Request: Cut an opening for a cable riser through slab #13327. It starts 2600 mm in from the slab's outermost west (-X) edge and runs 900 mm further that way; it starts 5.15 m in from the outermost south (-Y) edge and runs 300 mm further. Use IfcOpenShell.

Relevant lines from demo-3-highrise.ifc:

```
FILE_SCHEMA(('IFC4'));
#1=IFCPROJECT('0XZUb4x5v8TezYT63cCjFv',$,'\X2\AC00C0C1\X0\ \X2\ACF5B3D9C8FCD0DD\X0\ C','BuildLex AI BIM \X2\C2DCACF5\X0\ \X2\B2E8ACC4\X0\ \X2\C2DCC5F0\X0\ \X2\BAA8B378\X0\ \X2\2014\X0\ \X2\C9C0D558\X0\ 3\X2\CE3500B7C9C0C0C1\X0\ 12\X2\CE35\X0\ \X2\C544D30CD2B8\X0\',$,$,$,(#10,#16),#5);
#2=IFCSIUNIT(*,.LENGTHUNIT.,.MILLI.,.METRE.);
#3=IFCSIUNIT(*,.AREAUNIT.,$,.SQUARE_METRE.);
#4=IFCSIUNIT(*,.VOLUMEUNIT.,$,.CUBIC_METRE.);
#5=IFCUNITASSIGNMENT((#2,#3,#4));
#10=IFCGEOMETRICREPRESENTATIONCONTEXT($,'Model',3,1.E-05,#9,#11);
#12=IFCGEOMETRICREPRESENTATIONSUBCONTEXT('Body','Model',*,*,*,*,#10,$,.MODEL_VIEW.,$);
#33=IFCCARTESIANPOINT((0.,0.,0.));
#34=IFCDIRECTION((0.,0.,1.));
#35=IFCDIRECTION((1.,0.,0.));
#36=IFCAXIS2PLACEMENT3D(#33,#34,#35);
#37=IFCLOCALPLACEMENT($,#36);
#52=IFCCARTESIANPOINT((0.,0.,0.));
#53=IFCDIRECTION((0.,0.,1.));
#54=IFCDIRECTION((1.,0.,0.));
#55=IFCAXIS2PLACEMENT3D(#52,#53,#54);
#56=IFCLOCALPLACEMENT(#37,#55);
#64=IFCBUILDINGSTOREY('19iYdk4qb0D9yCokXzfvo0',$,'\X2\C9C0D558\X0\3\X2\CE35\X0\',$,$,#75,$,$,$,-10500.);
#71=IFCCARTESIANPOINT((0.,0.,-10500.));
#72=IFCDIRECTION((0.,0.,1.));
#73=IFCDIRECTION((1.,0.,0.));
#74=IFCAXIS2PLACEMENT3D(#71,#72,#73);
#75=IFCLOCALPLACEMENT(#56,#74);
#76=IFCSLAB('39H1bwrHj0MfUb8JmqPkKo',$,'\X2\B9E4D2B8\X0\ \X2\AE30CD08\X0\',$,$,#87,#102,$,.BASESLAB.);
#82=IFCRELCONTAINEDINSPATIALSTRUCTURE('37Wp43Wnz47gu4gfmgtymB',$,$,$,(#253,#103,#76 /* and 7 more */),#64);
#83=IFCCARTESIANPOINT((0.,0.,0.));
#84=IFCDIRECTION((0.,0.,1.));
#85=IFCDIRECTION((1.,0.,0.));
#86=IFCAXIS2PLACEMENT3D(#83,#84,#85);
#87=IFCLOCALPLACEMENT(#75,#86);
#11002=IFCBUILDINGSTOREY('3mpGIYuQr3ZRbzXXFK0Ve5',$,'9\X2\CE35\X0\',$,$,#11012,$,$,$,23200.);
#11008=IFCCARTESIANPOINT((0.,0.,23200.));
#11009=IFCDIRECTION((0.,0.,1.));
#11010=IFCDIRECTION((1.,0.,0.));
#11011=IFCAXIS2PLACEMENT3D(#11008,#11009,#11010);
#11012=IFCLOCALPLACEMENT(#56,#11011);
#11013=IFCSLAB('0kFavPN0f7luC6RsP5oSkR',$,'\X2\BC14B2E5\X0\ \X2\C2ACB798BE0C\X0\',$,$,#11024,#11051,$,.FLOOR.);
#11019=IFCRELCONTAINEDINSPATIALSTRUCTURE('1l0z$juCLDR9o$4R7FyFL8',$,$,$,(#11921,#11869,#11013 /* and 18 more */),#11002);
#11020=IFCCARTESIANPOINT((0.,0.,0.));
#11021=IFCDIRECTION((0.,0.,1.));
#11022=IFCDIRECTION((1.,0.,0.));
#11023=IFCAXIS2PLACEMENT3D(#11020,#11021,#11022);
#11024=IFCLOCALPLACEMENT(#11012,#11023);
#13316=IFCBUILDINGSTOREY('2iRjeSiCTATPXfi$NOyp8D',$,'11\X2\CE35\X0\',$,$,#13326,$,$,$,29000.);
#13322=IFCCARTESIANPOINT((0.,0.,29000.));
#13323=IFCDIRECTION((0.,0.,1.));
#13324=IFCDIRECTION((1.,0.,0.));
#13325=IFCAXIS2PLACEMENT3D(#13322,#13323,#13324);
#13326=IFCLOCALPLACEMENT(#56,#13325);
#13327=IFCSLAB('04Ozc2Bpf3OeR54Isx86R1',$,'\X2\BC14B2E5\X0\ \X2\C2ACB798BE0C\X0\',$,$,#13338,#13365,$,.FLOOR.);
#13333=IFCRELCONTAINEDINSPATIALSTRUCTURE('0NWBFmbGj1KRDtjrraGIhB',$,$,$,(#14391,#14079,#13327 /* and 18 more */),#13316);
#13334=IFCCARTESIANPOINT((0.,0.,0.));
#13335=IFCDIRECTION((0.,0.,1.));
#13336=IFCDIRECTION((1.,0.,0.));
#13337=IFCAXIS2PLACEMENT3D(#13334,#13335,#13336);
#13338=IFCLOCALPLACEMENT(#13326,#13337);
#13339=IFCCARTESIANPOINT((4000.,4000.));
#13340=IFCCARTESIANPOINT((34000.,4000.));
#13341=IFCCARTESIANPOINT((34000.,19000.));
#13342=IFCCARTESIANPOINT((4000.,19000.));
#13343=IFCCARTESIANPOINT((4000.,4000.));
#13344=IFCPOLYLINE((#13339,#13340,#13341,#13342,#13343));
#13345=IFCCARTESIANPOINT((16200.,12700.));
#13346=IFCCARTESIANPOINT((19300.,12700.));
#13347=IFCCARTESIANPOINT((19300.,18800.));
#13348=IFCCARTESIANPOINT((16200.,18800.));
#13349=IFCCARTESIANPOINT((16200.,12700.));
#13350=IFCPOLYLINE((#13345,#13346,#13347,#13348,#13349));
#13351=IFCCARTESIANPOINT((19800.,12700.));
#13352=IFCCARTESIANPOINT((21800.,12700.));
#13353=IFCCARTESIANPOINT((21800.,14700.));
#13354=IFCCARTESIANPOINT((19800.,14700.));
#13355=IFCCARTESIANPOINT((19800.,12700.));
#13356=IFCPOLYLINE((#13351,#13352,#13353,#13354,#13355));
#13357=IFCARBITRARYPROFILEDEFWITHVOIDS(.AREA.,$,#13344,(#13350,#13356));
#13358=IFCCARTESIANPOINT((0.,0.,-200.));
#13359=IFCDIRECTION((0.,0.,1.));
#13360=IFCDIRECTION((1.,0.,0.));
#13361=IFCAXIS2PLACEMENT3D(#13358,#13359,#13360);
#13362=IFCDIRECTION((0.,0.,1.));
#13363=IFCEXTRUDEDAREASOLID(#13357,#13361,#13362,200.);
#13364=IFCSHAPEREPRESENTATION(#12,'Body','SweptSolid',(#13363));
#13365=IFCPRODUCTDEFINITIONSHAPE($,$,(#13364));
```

```python
import numpy as np
import ifcopenshell
import ifcopenshell.api.feature
import ifcopenshell.api.geometry
import ifcopenshell.api.root
import ifcopenshell.geom
import ifcopenshell.util.placement
import ifcopenshell.util.representation
import ifcopenshell.util.shape
import ifcopenshell.util.unit

model = ifcopenshell.open("demo-3-highrise.ifc")
unit_scale = ifcopenshell.util.unit.calculate_unit_scale(model)
settings = ifcopenshell.geom.settings()


def volume(element):
    """Net volume in cubic metres, openings subtracted."""
    shape = ifcopenshell.geom.create_shape(settings, element)
    return ifcopenshell.util.shape.get_volume(shape.geometry)


slab = model.by_guid("04Ozc2Bpf3OeR54Isx86R1")
before = volume(slab)

# Extent in the slab's own axes, in metres. The edges named are its -X and -Y sides.
slab_shape = ifcopenshell.geom.create_shape(settings, slab)
vertices = ifcopenshell.util.shape.get_vertices(slab_shape.geometry)
x_min, y_min, bottom = vertices.min(axis=0)
top = vertices[:, 2].max()

opening = ifcopenshell.api.root.create_entity(model, ifc_class="IfcOpeningElement", name="Cable riser opening", predefined_type="OPENING")
context = ifcopenshell.util.representation.get_context(model, "Model", "Body", "MODEL_VIEW")
width, depth = 0.9, 0.3
outline = [(0.0, 0.0), (width, 0.0), (width, depth), (0.0, depth), (0.0, 0.0)]
# Overshoot both faces by 50 mm so the cut is clean.
shape = ifcopenshell.api.geometry.add_slab_representation(
    model, context=context, depth=top - bottom + 0.1, polyline=outline
)
ifcopenshell.api.geometry.assign_representation(model, product=opening, representation=shape)

matrix = ifcopenshell.util.placement.get_local_placement(slab.ObjectPlacement)
matrix[:, 3] = matrix @ np.append(np.array([x_min + 2.6, y_min + 5.15, bottom - 0.05]) / unit_scale, 1.0)
ifcopenshell.api.geometry.edit_object_placement(model, product=opening, matrix=matrix, is_si=False)
ifcopenshell.api.feature.add_feature(model, feature=opening, element=slab)

after = volume(slab)

print(f"slab volume {before:.3f} -> {after:.3f} m3")

model.write("demo-3-highrise_edited.ifc")
```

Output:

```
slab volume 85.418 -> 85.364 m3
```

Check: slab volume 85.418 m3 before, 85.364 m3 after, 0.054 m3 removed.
